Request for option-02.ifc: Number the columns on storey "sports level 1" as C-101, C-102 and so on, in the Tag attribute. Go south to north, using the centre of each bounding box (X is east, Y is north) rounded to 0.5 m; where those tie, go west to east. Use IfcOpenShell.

First a look at what the model holds.

```python
import ifcopenshell
import ifcopenshell.util.element
import ifcopenshell.util.placement

model = ifcopenshell.open("option-02.ifc")
print(model.schema)
storey = next(s for s in model.by_type("IfcBuildingStorey") if s.Name == "sports level 1")
columns = [e for e in ifcopenshell.util.element.get_decomposition(storey) if e.is_a("IfcColumn")]
for e in sorted(columns, key=lambda e: e.id()):
    origin = ifcopenshell.util.placement.get_local_placement(e.ObjectPlacement)[:3, 3]
    print(e.id(), e.Tag, e.Name, origin.round(2) + 0.0, sep=" | ")
```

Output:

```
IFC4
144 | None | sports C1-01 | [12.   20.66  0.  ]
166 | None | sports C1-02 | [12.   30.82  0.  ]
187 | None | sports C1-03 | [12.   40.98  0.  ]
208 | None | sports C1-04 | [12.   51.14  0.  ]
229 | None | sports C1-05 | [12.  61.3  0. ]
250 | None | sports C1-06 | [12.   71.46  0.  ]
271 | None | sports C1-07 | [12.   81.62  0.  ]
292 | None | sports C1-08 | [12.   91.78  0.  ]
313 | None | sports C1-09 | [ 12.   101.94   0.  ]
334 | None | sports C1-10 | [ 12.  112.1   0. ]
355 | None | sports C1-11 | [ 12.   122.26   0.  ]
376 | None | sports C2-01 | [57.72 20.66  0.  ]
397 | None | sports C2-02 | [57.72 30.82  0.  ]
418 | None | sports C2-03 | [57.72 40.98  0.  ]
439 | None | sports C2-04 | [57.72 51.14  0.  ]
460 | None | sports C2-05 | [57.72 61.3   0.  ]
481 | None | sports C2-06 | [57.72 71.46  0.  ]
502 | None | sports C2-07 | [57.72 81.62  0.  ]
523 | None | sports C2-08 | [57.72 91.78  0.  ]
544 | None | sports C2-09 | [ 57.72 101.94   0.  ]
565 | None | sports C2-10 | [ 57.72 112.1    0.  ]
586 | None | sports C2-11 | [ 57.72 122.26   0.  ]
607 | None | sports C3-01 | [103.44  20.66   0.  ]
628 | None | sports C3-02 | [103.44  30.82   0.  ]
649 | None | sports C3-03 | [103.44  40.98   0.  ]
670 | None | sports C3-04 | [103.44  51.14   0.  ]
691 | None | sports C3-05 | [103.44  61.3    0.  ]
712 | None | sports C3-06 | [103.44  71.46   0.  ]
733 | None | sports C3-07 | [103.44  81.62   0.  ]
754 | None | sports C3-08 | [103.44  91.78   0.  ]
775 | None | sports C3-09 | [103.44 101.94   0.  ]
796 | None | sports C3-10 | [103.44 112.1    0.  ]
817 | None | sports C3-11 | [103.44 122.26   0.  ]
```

```python
import ifcopenshell
import ifcopenshell.geom
import ifcopenshell.util.element
import ifcopenshell.util.shape

model = ifcopenshell.open("option-02.ifc")
settings = ifcopenshell.geom.settings()
settings.set("use-world-coords", True)


def centre(element):
    shape = ifcopenshell.geom.create_shape(settings, element)
    return ifcopenshell.util.shape.get_bbox_centroid(shape.geometry)


storey = next(s for s in model.by_type("IfcBuildingStorey") if s.Name == "sports level 1")
columns = [e for e in ifcopenshell.util.element.get_decomposition(storey) if e.is_a("IfcColumn")]

# Insertion points can sit at a corner or the storey origin, so sort by the geometry (in metres).
centres = {e: centre(e) for e in columns}
columns.sort(key=lambda e: (round(centres[e][1] / 0.5), centres[e][0]))

for i, e in enumerate(columns, start=1):
    number = f"C-1{i:02d}"
    e.Tag = number
    print(e.id(), number)

model.write("option-02_rev.ifc")
```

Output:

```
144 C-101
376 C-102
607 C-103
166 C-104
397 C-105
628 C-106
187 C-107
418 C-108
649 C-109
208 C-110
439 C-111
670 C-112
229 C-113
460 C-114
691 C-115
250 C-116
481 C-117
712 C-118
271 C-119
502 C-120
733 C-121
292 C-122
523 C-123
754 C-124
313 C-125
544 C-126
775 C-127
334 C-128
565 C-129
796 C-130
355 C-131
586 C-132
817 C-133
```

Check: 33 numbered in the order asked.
